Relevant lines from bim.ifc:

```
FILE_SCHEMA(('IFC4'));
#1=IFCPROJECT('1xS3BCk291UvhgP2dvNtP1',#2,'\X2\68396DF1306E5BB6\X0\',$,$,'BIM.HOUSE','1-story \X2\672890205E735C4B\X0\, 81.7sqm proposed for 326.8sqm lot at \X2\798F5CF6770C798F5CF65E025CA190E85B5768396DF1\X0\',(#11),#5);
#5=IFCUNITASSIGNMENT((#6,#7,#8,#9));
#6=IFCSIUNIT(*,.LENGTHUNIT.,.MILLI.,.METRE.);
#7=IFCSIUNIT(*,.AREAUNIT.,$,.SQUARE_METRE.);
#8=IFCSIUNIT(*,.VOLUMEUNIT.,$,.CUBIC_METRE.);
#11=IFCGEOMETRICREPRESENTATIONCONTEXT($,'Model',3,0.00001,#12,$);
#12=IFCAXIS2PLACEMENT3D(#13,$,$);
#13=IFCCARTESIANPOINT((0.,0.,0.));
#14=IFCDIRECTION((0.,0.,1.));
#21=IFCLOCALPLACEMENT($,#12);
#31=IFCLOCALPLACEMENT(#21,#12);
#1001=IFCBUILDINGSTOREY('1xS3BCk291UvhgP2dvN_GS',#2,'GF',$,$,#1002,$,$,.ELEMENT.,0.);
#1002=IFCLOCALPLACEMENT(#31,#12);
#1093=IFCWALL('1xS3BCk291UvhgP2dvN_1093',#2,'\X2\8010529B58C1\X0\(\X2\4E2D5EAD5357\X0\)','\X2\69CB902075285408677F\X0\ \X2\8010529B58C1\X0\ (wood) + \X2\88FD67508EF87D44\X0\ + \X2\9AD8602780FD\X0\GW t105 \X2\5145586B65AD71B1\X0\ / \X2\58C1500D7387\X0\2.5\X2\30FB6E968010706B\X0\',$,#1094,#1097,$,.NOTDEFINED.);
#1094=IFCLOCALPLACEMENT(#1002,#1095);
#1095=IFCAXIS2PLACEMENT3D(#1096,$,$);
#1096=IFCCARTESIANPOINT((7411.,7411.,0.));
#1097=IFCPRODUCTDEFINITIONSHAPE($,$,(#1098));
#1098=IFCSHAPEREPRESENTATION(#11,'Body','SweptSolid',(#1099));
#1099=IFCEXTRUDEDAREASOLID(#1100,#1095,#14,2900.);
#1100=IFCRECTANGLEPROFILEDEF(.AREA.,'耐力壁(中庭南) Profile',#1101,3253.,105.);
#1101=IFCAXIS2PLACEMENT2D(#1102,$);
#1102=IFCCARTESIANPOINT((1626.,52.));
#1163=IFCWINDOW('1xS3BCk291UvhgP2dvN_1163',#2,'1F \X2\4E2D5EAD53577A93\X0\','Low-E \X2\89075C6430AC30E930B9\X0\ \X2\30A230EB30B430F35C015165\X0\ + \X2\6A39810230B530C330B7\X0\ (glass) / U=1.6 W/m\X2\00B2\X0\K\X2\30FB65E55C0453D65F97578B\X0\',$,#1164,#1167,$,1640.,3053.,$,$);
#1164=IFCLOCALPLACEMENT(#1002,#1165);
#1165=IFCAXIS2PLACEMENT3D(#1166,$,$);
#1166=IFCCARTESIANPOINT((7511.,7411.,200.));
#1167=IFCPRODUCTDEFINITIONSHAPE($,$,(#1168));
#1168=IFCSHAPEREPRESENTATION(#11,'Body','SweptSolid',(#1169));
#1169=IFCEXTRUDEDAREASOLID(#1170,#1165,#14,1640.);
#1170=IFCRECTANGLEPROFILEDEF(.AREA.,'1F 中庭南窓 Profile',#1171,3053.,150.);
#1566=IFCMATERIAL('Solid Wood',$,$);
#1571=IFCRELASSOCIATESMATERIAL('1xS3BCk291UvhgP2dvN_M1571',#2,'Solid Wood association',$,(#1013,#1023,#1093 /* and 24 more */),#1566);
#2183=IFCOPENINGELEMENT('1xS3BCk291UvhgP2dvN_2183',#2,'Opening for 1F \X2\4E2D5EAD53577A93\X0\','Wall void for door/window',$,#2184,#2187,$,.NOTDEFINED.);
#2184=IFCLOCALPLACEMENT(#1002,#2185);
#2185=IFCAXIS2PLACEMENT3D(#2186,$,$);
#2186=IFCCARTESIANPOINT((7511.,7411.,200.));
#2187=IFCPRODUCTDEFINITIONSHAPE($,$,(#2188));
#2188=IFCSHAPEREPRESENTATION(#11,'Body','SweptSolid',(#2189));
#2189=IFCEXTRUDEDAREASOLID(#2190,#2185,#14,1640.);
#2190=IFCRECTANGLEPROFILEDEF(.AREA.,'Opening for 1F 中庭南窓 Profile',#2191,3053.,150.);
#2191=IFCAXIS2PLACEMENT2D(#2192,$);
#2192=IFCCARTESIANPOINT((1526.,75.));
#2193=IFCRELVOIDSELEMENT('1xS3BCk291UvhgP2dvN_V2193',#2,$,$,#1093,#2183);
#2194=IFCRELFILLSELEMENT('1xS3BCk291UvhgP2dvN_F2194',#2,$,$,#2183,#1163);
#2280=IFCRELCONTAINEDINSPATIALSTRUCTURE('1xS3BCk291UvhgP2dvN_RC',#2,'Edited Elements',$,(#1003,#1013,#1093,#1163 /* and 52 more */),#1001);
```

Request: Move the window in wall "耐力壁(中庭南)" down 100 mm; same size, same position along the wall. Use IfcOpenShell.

```python
import numpy as np
import ifcopenshell
import ifcopenshell.api.geometry
import ifcopenshell.util.placement
import ifcopenshell.util.unit

model = ifcopenshell.open("bim.ifc")
unit_scale = ifcopenshell.util.unit.calculate_unit_scale(model)

window = model.by_guid("1xS3BCk291UvhgP2dvN_1163")
opening = window.FillsVoids[0].RelatingOpeningElement
dz = -100.0

shift = np.array([0.0, 0.0, dz])
# The window is not placed relative to its opening, so move both.
for product in (opening, window):
    matrix = ifcopenshell.util.placement.get_local_placement(product.ObjectPlacement)
    matrix[:3, 3] += shift
    ifcopenshell.api.geometry.edit_object_placement(model, product=product, matrix=matrix, is_si=False)

print(f"moved by {dz * unit_scale:+.3f} m")

model.write("bim_v2.ifc")
```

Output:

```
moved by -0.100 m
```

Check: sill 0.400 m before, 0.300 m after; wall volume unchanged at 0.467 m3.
